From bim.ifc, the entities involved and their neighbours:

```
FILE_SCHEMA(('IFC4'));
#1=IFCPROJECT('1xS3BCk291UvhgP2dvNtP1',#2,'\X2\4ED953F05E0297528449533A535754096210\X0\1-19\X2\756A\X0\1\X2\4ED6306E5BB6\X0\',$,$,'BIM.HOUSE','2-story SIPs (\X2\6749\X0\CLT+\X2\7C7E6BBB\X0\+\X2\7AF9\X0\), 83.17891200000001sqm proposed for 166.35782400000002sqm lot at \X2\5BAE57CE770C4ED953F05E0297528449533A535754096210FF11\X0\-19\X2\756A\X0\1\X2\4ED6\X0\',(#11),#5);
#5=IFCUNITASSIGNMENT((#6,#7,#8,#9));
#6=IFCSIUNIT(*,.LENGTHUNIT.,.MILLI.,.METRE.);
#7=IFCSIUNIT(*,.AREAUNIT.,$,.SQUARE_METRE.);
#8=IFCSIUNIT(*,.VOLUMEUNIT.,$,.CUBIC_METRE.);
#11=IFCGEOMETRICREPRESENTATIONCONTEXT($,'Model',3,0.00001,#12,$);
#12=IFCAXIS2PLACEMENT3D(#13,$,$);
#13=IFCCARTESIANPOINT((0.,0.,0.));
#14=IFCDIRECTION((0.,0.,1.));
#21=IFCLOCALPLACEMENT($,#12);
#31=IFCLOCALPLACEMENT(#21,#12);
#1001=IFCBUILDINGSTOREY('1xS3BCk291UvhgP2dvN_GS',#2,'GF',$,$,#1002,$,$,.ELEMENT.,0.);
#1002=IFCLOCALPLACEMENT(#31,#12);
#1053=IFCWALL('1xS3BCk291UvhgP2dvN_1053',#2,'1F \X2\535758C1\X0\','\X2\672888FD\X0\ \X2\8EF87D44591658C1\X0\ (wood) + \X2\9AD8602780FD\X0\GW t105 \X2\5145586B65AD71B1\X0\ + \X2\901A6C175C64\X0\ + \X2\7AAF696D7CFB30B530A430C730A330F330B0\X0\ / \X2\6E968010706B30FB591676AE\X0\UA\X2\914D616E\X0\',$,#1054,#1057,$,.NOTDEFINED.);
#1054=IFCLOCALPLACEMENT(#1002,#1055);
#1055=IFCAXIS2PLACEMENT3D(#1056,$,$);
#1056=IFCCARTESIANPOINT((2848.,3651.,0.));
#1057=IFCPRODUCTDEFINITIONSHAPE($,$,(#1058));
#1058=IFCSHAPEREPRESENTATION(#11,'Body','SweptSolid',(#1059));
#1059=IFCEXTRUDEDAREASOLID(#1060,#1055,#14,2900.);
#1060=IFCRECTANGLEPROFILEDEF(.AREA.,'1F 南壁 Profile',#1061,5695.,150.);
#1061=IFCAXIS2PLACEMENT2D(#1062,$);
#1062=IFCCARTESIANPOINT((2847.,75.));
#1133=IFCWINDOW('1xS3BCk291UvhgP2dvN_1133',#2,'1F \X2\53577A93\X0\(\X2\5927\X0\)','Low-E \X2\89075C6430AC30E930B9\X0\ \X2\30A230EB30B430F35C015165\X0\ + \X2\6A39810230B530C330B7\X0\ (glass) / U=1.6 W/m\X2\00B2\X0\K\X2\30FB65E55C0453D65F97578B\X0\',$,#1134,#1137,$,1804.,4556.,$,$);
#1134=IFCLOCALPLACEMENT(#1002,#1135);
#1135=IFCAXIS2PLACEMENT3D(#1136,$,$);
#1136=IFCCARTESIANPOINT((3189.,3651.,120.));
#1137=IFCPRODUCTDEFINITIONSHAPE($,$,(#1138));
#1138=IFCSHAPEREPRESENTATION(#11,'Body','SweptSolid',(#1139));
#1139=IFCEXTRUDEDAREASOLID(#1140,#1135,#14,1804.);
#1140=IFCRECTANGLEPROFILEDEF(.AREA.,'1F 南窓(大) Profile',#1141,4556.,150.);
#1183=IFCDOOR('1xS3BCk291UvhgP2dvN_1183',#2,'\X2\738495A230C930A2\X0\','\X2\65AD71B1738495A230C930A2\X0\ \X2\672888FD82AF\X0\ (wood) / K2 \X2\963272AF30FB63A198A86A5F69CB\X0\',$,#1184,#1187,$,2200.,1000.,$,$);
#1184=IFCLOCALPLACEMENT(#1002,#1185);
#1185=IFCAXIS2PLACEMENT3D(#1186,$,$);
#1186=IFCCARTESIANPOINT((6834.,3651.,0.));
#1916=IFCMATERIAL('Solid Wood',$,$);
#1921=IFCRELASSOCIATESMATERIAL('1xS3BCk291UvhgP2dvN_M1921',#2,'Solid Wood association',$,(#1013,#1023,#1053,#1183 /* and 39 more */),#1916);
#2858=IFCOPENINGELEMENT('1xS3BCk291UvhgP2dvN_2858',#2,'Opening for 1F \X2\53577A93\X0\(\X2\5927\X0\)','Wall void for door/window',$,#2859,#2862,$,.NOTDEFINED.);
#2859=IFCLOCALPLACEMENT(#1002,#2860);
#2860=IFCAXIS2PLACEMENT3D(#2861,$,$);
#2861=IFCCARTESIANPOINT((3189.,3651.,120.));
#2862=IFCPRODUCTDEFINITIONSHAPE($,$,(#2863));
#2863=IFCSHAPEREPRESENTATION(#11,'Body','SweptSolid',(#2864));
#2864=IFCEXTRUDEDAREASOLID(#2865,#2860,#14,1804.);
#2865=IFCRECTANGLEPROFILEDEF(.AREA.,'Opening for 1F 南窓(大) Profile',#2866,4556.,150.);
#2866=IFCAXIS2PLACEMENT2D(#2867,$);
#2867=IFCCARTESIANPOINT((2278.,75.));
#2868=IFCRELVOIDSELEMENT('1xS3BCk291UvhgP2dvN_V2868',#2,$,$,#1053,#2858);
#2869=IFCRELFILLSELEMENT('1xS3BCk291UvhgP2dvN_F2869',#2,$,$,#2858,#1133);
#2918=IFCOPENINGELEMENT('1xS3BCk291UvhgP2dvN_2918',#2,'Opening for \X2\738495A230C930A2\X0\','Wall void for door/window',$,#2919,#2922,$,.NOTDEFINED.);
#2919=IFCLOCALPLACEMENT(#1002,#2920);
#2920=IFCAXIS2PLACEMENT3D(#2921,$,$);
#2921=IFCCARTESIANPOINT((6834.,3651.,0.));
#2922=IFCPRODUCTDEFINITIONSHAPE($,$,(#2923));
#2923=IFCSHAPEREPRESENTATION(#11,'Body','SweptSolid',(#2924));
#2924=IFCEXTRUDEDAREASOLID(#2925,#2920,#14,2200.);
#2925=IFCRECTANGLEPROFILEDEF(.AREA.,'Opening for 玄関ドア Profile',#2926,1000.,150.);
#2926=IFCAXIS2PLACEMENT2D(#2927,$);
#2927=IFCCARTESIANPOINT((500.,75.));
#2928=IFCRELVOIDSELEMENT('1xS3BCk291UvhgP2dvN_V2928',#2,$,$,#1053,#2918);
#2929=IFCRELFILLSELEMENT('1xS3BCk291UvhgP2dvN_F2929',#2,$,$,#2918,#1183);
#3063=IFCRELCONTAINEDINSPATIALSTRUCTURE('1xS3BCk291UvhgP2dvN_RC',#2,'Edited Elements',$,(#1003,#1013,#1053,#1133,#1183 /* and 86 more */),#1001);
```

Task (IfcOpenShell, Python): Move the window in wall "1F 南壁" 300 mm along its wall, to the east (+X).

```python
import ifcopenshell
import ifcopenshell.api.geometry
import ifcopenshell.util.placement
import ifcopenshell.util.unit

model = ifcopenshell.open("bim.ifc")
unit_scale = ifcopenshell.util.unit.calculate_unit_scale(model)

window = model.by_id(1133)
opening = window.FillsVoids[0].RelatingOpeningElement
wall = opening.VoidsElements[0].RelatingBuildingElement

wall_matrix = ifcopenshell.util.placement.get_local_placement(wall.ObjectPlacement)
shift = wall_matrix[:3, 0] * 0.3 / unit_scale
before = ifcopenshell.util.placement.get_local_placement(window.ObjectPlacement)[:3, 3].copy()

# The window is not placed relative to its opening, so move both.
for product in (opening, window):
    matrix = ifcopenshell.util.placement.get_local_placement(product.ObjectPlacement)
    matrix[:3, 3] += shift
    ifcopenshell.api.geometry.edit_object_placement(model, product=product, matrix=matrix, is_si=False)

after = ifcopenshell.util.placement.get_local_placement(window.ObjectPlacement)[:3, 3]
print("window moved by", (after - before).round(3) + 0.0)

model.write("bim-out.ifc")
```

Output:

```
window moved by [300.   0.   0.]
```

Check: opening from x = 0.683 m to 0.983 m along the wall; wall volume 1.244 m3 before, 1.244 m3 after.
